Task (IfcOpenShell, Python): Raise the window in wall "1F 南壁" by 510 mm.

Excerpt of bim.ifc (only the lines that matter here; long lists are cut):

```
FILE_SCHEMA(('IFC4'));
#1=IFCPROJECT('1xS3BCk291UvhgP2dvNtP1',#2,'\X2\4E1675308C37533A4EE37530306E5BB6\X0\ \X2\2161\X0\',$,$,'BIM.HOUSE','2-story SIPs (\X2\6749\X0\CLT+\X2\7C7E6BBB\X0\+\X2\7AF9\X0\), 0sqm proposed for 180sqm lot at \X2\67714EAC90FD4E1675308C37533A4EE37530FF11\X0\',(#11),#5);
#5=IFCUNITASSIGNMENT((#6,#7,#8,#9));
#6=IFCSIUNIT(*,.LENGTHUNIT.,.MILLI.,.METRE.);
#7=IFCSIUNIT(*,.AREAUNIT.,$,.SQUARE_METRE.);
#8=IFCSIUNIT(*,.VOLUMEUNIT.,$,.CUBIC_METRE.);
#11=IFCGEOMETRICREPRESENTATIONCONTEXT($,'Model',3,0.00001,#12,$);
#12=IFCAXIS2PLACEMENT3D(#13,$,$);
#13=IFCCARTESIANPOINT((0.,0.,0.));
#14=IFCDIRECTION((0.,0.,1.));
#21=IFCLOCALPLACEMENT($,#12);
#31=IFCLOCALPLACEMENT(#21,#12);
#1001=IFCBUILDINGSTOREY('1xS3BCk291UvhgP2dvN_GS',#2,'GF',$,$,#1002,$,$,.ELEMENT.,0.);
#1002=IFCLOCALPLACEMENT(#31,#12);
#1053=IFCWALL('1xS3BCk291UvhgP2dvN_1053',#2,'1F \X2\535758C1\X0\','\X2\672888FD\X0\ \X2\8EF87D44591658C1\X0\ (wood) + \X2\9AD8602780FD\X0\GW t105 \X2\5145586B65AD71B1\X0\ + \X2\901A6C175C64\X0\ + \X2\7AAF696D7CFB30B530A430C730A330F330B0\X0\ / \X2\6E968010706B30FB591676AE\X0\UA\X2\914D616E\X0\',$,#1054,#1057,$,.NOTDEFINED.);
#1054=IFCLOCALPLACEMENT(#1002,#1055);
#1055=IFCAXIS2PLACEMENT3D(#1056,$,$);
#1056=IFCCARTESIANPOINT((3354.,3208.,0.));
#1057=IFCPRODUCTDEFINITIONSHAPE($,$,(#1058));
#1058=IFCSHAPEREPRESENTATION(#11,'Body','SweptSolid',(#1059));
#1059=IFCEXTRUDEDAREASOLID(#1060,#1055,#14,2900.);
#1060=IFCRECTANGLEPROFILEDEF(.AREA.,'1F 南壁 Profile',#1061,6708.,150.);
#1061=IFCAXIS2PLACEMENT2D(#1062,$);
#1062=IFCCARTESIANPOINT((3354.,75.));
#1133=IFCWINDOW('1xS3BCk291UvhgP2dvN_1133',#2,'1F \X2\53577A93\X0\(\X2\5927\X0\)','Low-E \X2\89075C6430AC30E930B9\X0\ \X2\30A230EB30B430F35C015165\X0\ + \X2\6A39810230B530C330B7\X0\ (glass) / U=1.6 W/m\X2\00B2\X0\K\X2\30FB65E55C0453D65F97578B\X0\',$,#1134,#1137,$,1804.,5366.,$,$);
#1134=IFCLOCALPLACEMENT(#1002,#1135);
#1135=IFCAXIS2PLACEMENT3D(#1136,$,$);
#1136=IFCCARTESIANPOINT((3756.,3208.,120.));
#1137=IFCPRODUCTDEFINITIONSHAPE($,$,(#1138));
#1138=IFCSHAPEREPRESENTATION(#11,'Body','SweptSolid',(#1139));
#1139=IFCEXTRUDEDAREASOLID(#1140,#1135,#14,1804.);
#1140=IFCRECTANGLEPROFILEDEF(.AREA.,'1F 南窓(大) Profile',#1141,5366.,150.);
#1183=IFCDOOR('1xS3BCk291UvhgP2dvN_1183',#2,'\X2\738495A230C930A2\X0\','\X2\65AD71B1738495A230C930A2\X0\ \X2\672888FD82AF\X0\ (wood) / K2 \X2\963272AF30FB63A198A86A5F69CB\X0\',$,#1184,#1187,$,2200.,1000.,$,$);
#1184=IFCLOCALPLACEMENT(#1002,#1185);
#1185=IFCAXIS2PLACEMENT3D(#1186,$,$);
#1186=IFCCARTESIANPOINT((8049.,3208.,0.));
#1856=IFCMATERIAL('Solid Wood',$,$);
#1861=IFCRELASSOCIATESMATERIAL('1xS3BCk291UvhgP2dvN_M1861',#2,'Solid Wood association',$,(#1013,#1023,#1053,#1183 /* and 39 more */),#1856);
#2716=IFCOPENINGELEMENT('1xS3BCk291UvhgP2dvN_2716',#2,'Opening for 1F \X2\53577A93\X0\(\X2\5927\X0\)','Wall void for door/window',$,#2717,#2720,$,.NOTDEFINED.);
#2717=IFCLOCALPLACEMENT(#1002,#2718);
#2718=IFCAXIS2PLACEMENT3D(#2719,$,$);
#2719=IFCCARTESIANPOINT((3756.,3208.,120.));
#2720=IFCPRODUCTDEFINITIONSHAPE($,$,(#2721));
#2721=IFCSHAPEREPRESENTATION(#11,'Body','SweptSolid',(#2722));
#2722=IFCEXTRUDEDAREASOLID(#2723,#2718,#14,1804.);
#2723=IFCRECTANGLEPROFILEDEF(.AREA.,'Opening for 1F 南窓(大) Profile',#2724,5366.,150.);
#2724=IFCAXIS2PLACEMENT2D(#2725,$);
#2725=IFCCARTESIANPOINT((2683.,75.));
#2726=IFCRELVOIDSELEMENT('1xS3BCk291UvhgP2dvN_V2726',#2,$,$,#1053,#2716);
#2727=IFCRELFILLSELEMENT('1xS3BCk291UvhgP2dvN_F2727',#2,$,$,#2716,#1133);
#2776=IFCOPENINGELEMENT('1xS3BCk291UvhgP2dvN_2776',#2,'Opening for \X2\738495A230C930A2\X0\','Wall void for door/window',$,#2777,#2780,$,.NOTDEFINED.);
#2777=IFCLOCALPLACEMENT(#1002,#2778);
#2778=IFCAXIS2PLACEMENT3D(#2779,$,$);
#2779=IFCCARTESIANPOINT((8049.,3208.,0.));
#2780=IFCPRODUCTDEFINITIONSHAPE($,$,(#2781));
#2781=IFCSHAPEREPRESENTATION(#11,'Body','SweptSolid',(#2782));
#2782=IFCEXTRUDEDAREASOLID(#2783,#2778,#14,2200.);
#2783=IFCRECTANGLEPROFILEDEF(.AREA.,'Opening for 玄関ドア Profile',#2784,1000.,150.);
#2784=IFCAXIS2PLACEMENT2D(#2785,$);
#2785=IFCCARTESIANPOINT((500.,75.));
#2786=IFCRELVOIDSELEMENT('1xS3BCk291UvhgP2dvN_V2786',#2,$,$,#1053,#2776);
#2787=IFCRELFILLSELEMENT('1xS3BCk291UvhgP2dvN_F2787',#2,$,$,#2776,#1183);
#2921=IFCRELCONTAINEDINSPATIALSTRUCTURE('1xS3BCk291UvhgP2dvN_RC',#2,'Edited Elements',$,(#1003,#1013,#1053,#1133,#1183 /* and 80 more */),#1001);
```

```python
import numpy as np
import ifcopenshell
import ifcopenshell.api.geometry
import ifcopenshell.util.placement
import ifcopenshell.util.unit

model = ifcopenshell.open("bim.ifc")
unit_scale = ifcopenshell.util.unit.calculate_unit_scale(model)

window = model.by_id(1133)
opening = window.FillsVoids[0].RelatingOpeningElement
dz = 0.51 / unit_scale

shift = np.array([0.0, 0.0, dz])
# The window is not placed relative to its opening, so move both.
for product in (opening, window):
    matrix = ifcopenshell.util.placement.get_local_placement(product.ObjectPlacement)
    matrix[:3, 3] += shift
    ifcopenshell.api.geometry.edit_object_placement(model, product=product, matrix=matrix, is_si=False)

print(f"moved by {dz * unit_scale:+.3f} m")

model.write("bim_edited.ifc")
```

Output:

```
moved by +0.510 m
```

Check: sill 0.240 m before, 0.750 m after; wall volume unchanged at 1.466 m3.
